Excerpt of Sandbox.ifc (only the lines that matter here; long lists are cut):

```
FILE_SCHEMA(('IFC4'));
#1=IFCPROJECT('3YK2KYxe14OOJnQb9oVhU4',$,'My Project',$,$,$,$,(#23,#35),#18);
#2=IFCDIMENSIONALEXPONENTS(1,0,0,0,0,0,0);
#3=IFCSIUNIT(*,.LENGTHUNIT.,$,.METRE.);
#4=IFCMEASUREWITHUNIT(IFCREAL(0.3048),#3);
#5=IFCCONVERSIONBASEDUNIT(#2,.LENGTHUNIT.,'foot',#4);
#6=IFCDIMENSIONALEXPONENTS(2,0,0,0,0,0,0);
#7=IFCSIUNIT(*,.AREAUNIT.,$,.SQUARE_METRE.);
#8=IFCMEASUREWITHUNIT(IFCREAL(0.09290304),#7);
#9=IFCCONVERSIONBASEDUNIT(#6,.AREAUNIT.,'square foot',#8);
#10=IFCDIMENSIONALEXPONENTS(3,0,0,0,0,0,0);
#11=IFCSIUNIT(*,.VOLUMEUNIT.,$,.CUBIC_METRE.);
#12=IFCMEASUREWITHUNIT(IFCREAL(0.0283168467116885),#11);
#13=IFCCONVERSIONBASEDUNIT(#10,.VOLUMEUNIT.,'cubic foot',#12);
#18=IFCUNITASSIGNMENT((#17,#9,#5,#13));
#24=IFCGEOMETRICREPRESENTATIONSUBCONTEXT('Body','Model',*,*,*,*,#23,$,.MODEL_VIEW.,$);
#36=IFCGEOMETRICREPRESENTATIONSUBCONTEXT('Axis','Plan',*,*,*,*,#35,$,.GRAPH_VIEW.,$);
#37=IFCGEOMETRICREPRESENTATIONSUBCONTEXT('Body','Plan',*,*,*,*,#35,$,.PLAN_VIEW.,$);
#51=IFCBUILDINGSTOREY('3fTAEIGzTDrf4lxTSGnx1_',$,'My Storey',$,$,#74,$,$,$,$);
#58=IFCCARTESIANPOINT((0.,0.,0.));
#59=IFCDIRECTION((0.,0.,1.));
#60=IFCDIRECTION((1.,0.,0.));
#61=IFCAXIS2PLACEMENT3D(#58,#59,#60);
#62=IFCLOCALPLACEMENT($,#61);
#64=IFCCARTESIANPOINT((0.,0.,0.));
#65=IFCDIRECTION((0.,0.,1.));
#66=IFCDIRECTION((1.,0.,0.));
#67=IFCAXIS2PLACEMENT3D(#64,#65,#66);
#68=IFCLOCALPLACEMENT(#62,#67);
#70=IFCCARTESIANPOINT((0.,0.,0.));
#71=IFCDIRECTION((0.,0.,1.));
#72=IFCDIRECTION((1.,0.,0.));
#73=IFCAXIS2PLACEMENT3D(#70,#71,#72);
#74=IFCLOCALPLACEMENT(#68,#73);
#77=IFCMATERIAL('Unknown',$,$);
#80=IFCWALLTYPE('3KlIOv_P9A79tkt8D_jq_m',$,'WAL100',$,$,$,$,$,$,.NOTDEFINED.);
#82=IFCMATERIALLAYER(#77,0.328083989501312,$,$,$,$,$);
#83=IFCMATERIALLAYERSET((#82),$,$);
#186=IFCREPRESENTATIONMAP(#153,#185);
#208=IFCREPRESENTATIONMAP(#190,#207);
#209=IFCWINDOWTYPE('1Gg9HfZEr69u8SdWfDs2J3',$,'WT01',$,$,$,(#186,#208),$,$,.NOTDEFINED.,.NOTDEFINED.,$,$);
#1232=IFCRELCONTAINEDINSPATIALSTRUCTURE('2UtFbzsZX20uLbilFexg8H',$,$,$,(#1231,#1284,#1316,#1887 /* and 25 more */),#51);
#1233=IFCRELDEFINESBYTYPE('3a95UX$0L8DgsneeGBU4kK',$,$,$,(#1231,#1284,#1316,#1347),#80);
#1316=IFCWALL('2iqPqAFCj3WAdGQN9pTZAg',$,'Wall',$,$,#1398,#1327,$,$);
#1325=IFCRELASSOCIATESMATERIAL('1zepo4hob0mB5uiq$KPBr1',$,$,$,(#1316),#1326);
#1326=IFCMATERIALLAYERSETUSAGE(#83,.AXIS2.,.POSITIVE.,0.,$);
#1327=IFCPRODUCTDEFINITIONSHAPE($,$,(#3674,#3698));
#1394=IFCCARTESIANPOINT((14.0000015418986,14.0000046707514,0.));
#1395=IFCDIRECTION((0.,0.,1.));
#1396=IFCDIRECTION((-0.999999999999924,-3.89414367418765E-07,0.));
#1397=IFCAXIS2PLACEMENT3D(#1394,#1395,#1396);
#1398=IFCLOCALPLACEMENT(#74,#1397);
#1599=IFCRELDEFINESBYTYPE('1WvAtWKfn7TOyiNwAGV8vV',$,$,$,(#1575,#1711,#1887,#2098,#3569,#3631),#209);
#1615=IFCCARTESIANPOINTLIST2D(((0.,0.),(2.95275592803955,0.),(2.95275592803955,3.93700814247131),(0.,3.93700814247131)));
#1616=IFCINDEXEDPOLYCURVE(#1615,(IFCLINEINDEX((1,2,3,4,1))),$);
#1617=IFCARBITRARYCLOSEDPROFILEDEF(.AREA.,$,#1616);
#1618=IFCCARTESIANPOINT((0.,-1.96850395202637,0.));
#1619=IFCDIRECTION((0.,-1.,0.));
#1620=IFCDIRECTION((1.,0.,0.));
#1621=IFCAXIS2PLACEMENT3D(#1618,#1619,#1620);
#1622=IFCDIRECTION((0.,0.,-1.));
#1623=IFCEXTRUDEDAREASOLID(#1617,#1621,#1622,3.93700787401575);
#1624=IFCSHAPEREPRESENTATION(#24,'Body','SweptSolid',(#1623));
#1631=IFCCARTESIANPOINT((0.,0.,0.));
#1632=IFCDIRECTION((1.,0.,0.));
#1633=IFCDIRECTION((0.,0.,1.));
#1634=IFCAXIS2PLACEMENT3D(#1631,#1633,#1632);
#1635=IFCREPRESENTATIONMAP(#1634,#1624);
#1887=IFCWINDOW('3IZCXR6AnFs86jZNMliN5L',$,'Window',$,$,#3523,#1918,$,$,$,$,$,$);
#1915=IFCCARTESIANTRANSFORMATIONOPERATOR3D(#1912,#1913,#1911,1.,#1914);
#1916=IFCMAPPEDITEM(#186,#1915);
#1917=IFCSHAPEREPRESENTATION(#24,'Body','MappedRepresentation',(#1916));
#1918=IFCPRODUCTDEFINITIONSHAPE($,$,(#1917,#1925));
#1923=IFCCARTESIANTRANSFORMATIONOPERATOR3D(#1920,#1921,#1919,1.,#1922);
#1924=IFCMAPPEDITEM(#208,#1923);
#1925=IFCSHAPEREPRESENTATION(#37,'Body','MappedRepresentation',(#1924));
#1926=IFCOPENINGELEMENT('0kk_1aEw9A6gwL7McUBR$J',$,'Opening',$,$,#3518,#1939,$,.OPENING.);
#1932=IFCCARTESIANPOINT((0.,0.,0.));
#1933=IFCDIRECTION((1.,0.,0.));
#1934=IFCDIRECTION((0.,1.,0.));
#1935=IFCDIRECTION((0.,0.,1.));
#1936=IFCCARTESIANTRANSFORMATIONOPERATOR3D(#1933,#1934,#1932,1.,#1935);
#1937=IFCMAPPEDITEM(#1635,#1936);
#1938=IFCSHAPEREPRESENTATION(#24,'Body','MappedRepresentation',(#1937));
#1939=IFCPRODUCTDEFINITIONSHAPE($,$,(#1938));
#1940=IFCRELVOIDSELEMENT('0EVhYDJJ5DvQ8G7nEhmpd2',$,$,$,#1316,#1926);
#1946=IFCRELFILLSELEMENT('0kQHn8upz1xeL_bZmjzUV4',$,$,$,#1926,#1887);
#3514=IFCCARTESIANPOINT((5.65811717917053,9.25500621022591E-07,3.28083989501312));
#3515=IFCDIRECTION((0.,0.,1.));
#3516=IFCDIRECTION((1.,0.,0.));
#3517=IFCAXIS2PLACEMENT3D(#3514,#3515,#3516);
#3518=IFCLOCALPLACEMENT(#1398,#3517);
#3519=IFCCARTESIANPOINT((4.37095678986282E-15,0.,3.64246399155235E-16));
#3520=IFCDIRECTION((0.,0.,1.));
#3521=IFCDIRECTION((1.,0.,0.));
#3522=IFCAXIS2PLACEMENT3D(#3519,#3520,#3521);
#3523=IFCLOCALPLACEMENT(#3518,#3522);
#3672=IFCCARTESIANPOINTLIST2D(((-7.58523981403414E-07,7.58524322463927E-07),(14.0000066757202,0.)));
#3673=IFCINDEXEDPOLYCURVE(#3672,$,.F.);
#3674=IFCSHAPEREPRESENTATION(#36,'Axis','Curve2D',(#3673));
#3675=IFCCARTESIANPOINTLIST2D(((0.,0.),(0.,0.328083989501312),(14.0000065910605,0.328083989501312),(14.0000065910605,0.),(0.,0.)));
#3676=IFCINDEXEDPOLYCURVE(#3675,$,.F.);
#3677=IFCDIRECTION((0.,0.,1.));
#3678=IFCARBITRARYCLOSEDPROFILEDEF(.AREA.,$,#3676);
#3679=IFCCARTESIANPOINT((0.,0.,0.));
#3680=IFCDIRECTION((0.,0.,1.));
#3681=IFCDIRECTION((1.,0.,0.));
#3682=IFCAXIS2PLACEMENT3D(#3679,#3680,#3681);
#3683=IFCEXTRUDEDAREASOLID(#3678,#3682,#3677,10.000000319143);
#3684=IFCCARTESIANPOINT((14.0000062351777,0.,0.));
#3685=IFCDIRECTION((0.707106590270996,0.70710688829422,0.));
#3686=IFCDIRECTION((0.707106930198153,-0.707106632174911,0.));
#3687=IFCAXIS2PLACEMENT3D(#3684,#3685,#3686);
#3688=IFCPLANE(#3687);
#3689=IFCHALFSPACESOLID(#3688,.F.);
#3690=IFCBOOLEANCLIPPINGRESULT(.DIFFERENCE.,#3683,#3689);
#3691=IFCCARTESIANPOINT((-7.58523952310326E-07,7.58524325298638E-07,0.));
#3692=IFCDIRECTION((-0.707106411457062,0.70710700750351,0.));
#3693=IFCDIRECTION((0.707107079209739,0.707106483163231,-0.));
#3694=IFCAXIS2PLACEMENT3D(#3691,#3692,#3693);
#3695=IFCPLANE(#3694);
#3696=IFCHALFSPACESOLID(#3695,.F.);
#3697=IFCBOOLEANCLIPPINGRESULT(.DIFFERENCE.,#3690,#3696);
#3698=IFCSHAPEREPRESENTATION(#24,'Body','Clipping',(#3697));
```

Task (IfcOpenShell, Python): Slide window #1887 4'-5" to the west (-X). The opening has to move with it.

```python
import ifcopenshell
import ifcopenshell.api.geometry
import ifcopenshell.util.placement
import ifcopenshell.util.unit

model = ifcopenshell.open("Sandbox.ifc")
unit_scale = ifcopenshell.util.unit.calculate_unit_scale(model)

window = model.by_guid("3IZCXR6AnFs86jZNMliN5L")
opening = window.FillsVoids[0].RelatingOpeningElement
wall = opening.VoidsElements[0].RelatingBuildingElement

wall_matrix = ifcopenshell.util.placement.get_local_placement(wall.ObjectPlacement)
shift = wall_matrix[:3, 0] * 53 * 0.0254 / unit_scale
before = ifcopenshell.util.placement.get_local_placement(window.ObjectPlacement)[:3, 3].copy()

# The window is placed relative to its opening, so it follows when the opening moves.
matrix = ifcopenshell.util.placement.get_local_placement(opening.ObjectPlacement)
matrix[:3, 3] += shift
ifcopenshell.api.geometry.edit_object_placement(
    model, product=opening, matrix=matrix, is_si=False, should_transform_children=True
)

after = ifcopenshell.util.placement.get_local_placement(window.ObjectPlacement)[:3, 3]
print("window moved by", (after - before).round(3) + 0.0)

model.write("Sandbox_edited.ifc")
```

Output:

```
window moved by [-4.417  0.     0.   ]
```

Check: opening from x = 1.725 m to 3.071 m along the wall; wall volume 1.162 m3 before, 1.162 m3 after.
